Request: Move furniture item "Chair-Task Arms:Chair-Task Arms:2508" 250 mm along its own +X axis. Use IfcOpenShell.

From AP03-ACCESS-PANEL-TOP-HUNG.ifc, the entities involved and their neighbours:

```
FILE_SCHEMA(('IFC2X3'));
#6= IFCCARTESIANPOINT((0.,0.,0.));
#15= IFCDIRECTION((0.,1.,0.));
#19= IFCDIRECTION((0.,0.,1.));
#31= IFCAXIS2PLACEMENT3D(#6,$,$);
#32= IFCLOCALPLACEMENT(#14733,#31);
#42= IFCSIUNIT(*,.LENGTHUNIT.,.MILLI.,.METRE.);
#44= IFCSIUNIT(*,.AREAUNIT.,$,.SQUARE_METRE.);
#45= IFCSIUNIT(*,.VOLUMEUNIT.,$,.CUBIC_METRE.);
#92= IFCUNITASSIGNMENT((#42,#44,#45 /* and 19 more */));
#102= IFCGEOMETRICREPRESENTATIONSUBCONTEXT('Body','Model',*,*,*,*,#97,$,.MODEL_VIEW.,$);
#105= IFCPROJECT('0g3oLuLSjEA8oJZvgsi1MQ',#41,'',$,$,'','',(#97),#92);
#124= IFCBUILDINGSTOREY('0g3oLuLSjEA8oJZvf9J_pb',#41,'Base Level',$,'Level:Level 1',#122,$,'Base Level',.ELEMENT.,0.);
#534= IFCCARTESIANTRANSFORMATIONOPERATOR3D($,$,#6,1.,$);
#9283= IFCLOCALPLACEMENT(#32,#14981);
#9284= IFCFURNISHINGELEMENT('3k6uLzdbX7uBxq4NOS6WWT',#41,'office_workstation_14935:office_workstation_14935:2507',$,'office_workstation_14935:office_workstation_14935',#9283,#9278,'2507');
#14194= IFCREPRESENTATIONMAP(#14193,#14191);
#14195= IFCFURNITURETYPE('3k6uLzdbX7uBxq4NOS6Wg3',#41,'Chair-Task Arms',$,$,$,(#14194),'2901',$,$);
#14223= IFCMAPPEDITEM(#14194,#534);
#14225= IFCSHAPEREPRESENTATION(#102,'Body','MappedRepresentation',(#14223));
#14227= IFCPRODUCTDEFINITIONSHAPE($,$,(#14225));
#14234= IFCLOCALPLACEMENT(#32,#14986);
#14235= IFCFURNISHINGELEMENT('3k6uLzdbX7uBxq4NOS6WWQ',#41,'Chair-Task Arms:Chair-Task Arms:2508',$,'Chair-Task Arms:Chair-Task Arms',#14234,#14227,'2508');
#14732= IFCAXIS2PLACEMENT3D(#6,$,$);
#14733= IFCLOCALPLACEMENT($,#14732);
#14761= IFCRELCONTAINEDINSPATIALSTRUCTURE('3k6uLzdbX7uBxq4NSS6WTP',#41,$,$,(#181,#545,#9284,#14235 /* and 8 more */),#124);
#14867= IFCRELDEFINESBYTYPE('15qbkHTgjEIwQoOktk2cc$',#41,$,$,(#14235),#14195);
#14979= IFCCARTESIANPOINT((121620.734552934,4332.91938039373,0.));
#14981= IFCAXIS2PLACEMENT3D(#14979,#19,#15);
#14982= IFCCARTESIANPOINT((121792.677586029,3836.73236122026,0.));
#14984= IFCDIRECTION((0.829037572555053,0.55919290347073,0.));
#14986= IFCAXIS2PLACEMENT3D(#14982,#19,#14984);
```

```python
import ifcopenshell
import ifcopenshell.api.geometry
import ifcopenshell.util.placement
import ifcopenshell.util.unit

model = ifcopenshell.open("AP03-ACCESS-PANEL-TOP-HUNG.ifc")
unit_scale = ifcopenshell.util.unit.calculate_unit_scale(model)

item = model.by_id(14235)
matrix = ifcopenshell.util.placement.get_local_placement(item.ObjectPlacement)
matrix[:3, 3] += matrix[:3, 0] * 0.25 / unit_scale
ifcopenshell.api.geometry.edit_object_placement(model, product=item, matrix=matrix, is_si=False)

print(ifcopenshell.util.placement.get_local_placement(item.ObjectPlacement).round(3) + 0.0)

model.write("AP03-ACCESS-PANEL-TOP-HUNG_rev.ifc")
```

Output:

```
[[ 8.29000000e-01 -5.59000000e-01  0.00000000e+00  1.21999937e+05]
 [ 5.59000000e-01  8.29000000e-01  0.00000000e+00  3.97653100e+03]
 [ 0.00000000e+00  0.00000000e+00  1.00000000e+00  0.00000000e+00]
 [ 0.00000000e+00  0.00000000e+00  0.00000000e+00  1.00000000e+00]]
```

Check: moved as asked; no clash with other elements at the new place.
